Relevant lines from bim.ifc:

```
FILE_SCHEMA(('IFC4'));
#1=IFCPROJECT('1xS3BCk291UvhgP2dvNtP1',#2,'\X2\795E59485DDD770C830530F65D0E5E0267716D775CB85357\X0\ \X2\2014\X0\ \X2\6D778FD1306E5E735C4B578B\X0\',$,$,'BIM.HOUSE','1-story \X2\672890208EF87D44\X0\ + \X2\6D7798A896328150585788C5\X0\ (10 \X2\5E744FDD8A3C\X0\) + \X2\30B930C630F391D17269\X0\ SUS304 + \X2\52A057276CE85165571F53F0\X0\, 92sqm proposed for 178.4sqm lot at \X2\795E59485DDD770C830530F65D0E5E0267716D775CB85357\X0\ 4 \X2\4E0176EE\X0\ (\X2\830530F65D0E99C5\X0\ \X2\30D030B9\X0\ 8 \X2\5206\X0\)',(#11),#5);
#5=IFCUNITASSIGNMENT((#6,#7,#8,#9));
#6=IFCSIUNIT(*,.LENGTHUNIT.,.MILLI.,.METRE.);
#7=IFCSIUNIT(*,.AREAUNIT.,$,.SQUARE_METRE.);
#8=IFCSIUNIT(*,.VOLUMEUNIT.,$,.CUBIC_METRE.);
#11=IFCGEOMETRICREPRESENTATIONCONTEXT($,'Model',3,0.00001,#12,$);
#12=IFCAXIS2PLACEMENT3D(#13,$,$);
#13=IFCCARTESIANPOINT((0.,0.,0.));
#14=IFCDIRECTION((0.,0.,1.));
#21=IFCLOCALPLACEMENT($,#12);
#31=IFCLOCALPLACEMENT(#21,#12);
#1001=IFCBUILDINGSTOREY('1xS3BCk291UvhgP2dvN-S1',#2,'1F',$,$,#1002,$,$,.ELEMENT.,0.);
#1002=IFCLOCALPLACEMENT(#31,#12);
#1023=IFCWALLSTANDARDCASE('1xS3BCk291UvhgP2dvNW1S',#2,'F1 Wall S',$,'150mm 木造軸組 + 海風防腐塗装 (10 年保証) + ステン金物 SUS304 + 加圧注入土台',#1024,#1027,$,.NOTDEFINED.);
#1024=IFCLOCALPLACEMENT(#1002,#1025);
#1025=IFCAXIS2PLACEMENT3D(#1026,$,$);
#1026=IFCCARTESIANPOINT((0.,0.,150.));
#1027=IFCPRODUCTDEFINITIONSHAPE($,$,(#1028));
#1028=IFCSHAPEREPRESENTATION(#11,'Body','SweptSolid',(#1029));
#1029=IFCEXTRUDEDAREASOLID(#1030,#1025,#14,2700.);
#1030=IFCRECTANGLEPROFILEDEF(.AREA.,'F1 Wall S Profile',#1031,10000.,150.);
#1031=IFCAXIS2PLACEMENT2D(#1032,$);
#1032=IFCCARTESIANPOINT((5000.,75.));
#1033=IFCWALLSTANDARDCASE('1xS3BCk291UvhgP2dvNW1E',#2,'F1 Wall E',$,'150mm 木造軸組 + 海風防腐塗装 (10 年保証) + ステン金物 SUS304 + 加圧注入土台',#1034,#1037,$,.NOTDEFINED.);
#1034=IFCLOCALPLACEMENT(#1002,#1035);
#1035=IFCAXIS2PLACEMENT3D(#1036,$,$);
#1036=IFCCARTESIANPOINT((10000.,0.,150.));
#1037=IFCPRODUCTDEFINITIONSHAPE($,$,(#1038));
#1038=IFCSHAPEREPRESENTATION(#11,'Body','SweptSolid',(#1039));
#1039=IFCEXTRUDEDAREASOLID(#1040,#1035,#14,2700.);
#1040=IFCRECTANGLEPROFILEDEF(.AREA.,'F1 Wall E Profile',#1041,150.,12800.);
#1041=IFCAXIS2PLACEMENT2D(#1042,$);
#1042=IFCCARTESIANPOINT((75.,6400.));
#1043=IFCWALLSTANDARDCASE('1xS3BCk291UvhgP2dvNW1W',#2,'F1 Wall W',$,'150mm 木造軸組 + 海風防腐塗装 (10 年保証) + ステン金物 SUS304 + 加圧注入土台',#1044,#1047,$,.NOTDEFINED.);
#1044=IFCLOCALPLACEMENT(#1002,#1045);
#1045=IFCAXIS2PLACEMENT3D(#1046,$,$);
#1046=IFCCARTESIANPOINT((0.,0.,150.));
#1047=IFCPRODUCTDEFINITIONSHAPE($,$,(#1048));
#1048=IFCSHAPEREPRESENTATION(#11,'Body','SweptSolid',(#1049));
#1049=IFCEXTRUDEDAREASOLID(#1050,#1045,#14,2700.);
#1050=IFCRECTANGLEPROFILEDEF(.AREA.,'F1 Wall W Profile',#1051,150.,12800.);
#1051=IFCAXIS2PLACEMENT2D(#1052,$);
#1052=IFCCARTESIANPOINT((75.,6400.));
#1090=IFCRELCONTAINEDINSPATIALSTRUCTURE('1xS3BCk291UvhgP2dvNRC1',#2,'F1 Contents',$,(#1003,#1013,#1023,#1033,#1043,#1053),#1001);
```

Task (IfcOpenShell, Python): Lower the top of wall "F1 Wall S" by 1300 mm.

```python
import ifcopenshell
import ifcopenshell.geom
import ifcopenshell.util.shape
import ifcopenshell.util.unit

model = ifcopenshell.open("bim.ifc")
unit_scale = ifcopenshell.util.unit.calculate_unit_scale(model)
settings = ifcopenshell.geom.settings()


def volume(element):
    """Net volume in cubic metres, openings subtracted."""
    shape = ifcopenshell.geom.create_shape(settings, element)
    return ifcopenshell.util.shape.get_volume(shape.geometry)


wall = model.by_guid("1xS3BCk291UvhgP2dvNW1S")
before = volume(wall)

body = next(r for r in wall.Representation.Representations if r.RepresentationIdentifier == "Body")
solid = body.Items[0]
old_height = solid.Depth
solid.Depth -= 1.3 / unit_scale
after = volume(wall)

print(f"height {old_height:g} -> {solid.Depth:g}, volume {before:.3f} -> {after:.3f} m3")

model.write("bim_edited.ifc")
```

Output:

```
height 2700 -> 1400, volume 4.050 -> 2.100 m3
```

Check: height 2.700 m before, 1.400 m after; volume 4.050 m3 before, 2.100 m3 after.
